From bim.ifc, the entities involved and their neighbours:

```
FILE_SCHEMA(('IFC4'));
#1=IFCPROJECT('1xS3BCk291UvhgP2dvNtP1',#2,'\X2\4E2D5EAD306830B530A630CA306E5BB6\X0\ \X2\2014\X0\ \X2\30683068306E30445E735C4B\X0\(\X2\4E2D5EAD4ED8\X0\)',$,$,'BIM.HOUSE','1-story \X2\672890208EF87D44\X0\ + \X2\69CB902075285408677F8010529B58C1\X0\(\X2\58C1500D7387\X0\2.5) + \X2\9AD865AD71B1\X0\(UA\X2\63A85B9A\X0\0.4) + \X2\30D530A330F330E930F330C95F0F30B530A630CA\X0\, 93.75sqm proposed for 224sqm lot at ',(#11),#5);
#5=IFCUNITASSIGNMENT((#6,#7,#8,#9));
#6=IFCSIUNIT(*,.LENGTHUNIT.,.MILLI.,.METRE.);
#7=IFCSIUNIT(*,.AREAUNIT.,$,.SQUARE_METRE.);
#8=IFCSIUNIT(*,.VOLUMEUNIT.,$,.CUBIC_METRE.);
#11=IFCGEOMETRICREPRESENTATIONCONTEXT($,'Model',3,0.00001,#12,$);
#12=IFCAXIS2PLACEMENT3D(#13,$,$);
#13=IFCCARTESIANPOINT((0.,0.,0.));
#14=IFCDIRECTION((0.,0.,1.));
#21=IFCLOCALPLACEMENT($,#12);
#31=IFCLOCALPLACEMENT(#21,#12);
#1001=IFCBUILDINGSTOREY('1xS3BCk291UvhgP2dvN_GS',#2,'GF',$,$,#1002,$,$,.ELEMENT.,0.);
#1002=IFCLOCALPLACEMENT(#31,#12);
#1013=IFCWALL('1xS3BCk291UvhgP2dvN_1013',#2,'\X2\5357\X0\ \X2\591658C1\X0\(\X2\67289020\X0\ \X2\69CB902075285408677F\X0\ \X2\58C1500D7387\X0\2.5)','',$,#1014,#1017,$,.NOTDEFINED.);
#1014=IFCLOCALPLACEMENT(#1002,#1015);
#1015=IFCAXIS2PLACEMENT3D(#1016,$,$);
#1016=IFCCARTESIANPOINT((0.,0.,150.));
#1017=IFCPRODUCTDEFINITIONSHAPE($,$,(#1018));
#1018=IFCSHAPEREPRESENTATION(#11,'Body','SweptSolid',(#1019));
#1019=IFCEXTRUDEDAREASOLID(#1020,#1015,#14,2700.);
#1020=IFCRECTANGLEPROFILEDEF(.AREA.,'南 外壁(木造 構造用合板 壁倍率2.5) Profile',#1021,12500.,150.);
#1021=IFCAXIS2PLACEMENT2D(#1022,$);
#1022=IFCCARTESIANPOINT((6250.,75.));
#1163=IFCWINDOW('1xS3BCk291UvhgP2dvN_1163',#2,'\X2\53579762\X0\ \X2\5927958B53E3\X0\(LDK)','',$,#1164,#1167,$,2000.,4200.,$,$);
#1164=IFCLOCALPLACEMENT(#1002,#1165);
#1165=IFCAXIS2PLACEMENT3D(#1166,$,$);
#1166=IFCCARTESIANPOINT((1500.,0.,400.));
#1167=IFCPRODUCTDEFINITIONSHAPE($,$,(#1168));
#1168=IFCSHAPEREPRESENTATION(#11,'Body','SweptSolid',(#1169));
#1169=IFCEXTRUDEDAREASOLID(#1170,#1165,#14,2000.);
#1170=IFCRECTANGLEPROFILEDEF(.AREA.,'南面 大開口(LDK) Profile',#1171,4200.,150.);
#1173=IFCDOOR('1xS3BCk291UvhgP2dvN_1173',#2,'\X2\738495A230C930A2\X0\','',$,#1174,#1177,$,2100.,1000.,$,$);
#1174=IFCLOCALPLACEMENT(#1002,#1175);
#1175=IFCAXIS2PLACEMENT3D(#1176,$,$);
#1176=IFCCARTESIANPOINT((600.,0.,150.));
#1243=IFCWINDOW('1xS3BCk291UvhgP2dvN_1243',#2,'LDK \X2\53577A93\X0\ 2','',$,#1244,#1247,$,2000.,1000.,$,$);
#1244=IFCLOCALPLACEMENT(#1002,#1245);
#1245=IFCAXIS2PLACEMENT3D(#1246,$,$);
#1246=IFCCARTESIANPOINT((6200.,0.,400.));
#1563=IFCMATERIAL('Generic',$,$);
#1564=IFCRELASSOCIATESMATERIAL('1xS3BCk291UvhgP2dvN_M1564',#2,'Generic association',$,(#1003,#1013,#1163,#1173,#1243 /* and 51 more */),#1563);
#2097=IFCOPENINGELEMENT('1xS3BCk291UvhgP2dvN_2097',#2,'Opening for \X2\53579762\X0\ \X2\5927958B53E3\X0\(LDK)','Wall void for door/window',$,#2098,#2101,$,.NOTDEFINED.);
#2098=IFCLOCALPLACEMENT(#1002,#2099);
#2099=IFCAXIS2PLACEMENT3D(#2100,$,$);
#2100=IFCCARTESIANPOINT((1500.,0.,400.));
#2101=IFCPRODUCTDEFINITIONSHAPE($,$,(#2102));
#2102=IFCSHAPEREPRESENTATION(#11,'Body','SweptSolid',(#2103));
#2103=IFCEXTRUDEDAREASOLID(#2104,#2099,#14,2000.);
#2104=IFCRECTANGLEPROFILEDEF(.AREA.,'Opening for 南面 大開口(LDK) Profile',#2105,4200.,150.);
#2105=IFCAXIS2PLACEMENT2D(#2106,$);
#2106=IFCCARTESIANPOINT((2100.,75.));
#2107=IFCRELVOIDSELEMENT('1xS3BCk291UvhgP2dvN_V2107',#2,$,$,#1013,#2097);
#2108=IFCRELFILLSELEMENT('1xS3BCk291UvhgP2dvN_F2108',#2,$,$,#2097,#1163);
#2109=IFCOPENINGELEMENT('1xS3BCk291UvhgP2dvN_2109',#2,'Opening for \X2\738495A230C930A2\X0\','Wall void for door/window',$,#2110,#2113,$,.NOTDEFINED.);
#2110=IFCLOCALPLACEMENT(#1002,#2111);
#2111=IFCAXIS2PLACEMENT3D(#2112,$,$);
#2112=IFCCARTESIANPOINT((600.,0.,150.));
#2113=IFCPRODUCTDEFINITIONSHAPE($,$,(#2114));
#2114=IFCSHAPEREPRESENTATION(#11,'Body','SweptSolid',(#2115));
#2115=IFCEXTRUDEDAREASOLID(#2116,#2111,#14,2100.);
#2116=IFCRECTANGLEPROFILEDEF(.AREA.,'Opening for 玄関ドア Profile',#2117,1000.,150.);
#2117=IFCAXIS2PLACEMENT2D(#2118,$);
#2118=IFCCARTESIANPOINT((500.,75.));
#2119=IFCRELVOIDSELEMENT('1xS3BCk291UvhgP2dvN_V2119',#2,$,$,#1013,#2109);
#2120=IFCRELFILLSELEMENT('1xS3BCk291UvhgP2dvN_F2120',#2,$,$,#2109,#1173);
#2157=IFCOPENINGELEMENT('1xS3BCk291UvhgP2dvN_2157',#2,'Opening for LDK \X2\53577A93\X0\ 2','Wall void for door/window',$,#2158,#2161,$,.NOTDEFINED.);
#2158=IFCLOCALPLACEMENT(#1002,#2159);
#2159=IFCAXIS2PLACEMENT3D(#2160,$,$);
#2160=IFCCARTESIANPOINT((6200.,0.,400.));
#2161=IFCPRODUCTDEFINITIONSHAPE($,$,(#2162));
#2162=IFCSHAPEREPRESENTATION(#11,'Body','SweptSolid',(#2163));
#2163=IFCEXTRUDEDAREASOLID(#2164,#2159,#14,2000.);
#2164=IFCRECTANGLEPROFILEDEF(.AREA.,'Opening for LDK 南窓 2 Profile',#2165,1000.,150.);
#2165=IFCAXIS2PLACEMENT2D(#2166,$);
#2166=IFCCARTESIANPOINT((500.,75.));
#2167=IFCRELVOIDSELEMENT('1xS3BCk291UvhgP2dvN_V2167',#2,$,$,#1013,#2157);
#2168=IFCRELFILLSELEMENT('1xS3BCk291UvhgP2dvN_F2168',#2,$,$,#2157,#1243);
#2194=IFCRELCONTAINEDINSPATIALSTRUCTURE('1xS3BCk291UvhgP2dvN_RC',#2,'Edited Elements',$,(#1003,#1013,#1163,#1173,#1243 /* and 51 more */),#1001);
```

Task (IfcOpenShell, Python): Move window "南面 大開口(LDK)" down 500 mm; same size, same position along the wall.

```python
import numpy as np
import ifcopenshell
import ifcopenshell.api.geometry
import ifcopenshell.util.placement
import ifcopenshell.util.unit

model = ifcopenshell.open("bim.ifc")
unit_scale = ifcopenshell.util.unit.calculate_unit_scale(model)

window = model.by_guid("1xS3BCk291UvhgP2dvN_1163")
opening = window.FillsVoids[0].RelatingOpeningElement
dz = -0.5 / unit_scale

shift = np.array([0.0, 0.0, dz])
# The window is not placed relative to its opening, so move both.
for product in (opening, window):
    matrix = ifcopenshell.util.placement.get_local_placement(product.ObjectPlacement)
    matrix[:3, 3] += shift
    ifcopenshell.api.geometry.edit_object_placement(model, product=product, matrix=matrix, is_si=False)

print(f"moved by {dz * unit_scale:+.3f} m")

model.write("bim-out.ifc")
```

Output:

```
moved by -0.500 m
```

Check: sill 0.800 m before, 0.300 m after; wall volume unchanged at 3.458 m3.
